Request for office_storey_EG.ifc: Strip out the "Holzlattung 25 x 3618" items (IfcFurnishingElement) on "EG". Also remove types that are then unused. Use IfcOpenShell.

First a look at what the model holds.

```python
import ifcopenshell
import ifcopenshell.util.element

model = ifcopenshell.open("office_storey_EG.ifc")
print(model.schema)
storey = next(s for s in model.by_type("IfcBuildingStorey") if s.Name == "EG")
furniture = [e for e in ifcopenshell.util.element.get_decomposition(storey) if e.is_a("IfcFurnishingElement")]
seen = {}
for e in furniture:
    element_type = ifcopenshell.util.element.get_type(e)
    name = element_type.Name if element_type not in (None, e) else None
    seen[name] = seen.get(name, 0) + 1
for name, count in sorted(seen.items(), key=str):
    print(count, "x", name)
```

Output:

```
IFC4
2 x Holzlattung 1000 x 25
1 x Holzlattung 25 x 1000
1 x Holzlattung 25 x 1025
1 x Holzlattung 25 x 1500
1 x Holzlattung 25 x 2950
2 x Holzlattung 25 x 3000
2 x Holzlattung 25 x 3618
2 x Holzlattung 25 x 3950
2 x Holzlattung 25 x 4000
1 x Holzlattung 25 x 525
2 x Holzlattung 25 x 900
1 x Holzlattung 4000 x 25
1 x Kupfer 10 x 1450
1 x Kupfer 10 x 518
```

```python
import ifcopenshell
import ifcopenshell.api.root
import ifcopenshell.util.element

model = ifcopenshell.open("office_storey_EG.ifc")

storey = next(s for s in model.by_type("IfcBuildingStorey") if s.Name == "EG")
furniture = [e for e in ifcopenshell.util.element.get_decomposition(storey) if e.is_a("IfcFurnishingElement")]
targets = [e for e in furniture if (t := ifcopenshell.util.element.get_type(e)) not in (None, e) and t.Name == "Holzlattung 25 x 3618"]
types = {ifcopenshell.util.element.get_type(e) for e in targets} - {None, *targets}

for e in targets:
    ifcopenshell.api.root.remove_product(model, product=e)
print(len(targets), "removed")

unused = [t for t in types if not ifcopenshell.util.element.get_types(t)]
for t in unused:
    ifcopenshell.api.root.remove_product(model, product=t)
print(len(unused), "unused types removed")

model.write("office_storey_EG_rev.ifc")
```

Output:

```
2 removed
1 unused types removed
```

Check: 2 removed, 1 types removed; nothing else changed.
